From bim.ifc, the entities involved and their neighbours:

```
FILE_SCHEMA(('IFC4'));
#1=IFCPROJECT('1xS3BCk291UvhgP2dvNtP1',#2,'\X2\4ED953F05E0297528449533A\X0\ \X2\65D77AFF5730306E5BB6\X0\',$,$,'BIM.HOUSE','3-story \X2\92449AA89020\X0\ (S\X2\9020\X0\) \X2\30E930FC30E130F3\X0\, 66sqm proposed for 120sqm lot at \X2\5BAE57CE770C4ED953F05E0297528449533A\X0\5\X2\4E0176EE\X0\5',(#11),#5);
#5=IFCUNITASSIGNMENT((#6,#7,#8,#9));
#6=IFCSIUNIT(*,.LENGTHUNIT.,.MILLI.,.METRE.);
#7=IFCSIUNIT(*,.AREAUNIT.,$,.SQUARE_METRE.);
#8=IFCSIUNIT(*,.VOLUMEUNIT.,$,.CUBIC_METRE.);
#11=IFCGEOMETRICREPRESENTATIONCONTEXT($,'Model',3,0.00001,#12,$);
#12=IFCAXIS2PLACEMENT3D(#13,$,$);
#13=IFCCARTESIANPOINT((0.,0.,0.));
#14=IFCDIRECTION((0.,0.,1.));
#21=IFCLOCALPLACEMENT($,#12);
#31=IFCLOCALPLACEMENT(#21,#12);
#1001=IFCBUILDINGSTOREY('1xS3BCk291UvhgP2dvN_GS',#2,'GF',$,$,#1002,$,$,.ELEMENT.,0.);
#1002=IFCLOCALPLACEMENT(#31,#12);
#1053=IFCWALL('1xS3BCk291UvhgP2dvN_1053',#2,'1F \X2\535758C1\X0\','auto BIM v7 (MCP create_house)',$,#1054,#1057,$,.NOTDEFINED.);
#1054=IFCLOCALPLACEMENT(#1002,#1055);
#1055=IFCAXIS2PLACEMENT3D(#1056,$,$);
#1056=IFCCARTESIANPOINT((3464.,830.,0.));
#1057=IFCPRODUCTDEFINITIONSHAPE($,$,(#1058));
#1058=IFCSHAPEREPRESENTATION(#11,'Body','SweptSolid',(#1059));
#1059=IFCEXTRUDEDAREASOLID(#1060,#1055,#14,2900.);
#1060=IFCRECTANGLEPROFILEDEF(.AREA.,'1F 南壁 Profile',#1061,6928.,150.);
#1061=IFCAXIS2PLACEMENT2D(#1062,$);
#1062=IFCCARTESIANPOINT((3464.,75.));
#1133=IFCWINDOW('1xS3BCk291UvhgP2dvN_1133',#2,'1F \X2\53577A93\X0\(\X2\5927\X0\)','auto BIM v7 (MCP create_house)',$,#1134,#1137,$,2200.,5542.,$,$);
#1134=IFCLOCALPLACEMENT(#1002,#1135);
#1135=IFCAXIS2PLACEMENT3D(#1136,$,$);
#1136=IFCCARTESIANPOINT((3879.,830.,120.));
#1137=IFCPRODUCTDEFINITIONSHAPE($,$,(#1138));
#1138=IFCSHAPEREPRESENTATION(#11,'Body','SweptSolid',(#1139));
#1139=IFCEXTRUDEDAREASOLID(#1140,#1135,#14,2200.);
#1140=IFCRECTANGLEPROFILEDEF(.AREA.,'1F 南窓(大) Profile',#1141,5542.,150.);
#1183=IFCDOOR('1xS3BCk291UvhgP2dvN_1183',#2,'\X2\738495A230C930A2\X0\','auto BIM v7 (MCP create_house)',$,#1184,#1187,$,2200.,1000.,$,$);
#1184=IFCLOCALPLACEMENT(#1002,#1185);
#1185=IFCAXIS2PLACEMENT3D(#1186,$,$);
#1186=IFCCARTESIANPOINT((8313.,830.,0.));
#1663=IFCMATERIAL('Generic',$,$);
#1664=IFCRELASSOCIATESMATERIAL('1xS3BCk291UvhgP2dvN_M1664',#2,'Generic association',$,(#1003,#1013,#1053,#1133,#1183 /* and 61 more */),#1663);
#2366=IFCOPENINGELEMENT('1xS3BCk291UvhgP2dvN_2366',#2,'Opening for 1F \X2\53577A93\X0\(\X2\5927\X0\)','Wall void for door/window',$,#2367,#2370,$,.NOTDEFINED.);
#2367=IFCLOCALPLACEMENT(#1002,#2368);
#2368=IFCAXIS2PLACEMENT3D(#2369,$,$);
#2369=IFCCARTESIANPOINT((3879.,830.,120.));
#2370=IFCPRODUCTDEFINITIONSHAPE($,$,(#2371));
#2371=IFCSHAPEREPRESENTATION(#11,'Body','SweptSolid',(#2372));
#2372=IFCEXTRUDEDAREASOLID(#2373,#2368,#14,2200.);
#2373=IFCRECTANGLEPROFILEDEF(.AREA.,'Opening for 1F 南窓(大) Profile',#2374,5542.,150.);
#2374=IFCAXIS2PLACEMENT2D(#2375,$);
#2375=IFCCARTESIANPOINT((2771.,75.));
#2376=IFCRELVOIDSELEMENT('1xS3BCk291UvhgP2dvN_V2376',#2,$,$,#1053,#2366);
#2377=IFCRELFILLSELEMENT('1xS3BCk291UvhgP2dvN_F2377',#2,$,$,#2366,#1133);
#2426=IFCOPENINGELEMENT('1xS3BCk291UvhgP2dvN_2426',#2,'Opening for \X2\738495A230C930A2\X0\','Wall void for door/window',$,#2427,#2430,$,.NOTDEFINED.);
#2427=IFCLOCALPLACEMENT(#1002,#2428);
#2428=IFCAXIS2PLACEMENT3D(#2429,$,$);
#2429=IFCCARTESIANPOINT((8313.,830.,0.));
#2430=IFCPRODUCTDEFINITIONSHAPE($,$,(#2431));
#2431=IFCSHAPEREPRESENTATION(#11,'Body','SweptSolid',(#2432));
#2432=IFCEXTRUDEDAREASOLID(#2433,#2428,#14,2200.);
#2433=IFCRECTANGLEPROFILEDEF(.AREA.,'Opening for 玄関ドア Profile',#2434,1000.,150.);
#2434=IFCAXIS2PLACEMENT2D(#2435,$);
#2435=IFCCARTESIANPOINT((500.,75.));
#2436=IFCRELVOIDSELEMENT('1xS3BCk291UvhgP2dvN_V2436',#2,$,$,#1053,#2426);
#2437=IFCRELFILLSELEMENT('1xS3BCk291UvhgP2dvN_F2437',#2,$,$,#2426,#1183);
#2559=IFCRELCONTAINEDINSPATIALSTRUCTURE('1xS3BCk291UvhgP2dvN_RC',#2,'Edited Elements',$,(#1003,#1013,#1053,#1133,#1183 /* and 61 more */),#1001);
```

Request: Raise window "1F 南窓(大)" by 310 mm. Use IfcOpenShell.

```python
import numpy as np
import ifcopenshell
import ifcopenshell.api.geometry
import ifcopenshell.util.placement
import ifcopenshell.util.unit

model = ifcopenshell.open("bim.ifc")
unit_scale = ifcopenshell.util.unit.calculate_unit_scale(model)

window = model.by_guid("1xS3BCk291UvhgP2dvN_1133")
opening = window.FillsVoids[0].RelatingOpeningElement
dz = 0.31 / unit_scale

shift = np.array([0.0, 0.0, dz])
# The window is not placed relative to its opening, so move both.
for product in (opening, window):
    matrix = ifcopenshell.util.placement.get_local_placement(product.ObjectPlacement)
    matrix[:3, 3] += shift
    ifcopenshell.api.geometry.edit_object_placement(model, product=product, matrix=matrix, is_si=False)

print(f"moved by {dz * unit_scale:+.3f} m")

model.write("bim_rev.ifc")
```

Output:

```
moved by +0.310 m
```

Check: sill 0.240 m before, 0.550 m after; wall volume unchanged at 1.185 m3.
